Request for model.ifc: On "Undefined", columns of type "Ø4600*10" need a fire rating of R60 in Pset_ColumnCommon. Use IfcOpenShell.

First a look at what the model holds.

```python
import ifcopenshell
import ifcopenshell.util.element

model = ifcopenshell.open("model.ifc")
print(model.schema)
storey = next(s for s in model.by_type("IfcBuildingStorey") if s.Name == "Undefined")
columns = [e for e in ifcopenshell.util.element.get_decomposition(storey) if e.is_a("IfcColumn")]
seen = {}
for e in columns:
    element_type = ifcopenshell.util.element.get_type(e)
    key = (element_type.Name if element_type != e and element_type else None, ifcopenshell.util.element.get_pset(e, "Pset_ColumnCommon", "FireRating"))
    seen[key] = seen.get(key, 0) + 1
for (name, value), count in sorted(seen.items(), key=str):
    print(count, "x", name, "|", value)
```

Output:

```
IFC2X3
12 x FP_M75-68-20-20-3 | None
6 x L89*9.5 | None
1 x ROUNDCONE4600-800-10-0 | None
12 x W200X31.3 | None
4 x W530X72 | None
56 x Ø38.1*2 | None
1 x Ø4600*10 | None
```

```python
import ifcopenshell
import ifcopenshell.api.pset
import ifcopenshell.util.element

model = ifcopenshell.open("model.ifc")

storey = next(s for s in model.by_type("IfcBuildingStorey") if s.Name == "Undefined")
columns = [e for e in ifcopenshell.util.element.get_decomposition(storey) if e.is_a("IfcColumn")]

count = 0
for e in columns:
    element_type = ifcopenshell.util.element.get_type(e)
    if element_type in (None, e) or element_type.Name != "Ø4600*10":
        continue
    # add_pset returns the element's existing set when there is one.
    pset = ifcopenshell.api.pset.add_pset(model, product=e, name="Pset_ColumnCommon")
    ifcopenshell.api.pset.edit_pset(model, pset=pset, properties={"FireRating": "R60"})
    count += 1

print(count, "columns updated")

model.write("model-out.ifc")
```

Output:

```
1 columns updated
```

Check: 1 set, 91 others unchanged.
